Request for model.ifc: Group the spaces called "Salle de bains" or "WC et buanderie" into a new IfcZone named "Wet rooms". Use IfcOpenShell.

First a look at what the model holds.

```python
import ifcopenshell

model = ifcopenshell.open("model.ifc")
print(model.schema)
seen = {}
for space in model.by_type("IfcSpace"):
    seen[space.LongName] = seen.get(space.LongName, 0) + 1
for name, count in sorted(seen.items(), key=str):
    print(count, "x", name)
print("zones:", [z.Name for z in model.by_type("IfcZone")][:20])
```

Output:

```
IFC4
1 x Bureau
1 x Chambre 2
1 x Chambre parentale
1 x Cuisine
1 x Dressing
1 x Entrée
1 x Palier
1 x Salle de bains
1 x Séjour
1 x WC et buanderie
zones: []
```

```python
import ifcopenshell
import ifcopenshell.api.group
import ifcopenshell.api.root

model = ifcopenshell.open("model.ifc")

names = {"Salle de bains", "WC et buanderie"}
spaces = [s for s in model.by_type("IfcSpace") if s.LongName in names]

zone = ifcopenshell.api.root.create_entity(model, ifc_class="IfcZone", name="Wet rooms")
ifcopenshell.api.group.assign_group(model, products=spaces, group=zone)
print(len(spaces), "spaces in", zone.Name)

model.write("model-out.ifc")
```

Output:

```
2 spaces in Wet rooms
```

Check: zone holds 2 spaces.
